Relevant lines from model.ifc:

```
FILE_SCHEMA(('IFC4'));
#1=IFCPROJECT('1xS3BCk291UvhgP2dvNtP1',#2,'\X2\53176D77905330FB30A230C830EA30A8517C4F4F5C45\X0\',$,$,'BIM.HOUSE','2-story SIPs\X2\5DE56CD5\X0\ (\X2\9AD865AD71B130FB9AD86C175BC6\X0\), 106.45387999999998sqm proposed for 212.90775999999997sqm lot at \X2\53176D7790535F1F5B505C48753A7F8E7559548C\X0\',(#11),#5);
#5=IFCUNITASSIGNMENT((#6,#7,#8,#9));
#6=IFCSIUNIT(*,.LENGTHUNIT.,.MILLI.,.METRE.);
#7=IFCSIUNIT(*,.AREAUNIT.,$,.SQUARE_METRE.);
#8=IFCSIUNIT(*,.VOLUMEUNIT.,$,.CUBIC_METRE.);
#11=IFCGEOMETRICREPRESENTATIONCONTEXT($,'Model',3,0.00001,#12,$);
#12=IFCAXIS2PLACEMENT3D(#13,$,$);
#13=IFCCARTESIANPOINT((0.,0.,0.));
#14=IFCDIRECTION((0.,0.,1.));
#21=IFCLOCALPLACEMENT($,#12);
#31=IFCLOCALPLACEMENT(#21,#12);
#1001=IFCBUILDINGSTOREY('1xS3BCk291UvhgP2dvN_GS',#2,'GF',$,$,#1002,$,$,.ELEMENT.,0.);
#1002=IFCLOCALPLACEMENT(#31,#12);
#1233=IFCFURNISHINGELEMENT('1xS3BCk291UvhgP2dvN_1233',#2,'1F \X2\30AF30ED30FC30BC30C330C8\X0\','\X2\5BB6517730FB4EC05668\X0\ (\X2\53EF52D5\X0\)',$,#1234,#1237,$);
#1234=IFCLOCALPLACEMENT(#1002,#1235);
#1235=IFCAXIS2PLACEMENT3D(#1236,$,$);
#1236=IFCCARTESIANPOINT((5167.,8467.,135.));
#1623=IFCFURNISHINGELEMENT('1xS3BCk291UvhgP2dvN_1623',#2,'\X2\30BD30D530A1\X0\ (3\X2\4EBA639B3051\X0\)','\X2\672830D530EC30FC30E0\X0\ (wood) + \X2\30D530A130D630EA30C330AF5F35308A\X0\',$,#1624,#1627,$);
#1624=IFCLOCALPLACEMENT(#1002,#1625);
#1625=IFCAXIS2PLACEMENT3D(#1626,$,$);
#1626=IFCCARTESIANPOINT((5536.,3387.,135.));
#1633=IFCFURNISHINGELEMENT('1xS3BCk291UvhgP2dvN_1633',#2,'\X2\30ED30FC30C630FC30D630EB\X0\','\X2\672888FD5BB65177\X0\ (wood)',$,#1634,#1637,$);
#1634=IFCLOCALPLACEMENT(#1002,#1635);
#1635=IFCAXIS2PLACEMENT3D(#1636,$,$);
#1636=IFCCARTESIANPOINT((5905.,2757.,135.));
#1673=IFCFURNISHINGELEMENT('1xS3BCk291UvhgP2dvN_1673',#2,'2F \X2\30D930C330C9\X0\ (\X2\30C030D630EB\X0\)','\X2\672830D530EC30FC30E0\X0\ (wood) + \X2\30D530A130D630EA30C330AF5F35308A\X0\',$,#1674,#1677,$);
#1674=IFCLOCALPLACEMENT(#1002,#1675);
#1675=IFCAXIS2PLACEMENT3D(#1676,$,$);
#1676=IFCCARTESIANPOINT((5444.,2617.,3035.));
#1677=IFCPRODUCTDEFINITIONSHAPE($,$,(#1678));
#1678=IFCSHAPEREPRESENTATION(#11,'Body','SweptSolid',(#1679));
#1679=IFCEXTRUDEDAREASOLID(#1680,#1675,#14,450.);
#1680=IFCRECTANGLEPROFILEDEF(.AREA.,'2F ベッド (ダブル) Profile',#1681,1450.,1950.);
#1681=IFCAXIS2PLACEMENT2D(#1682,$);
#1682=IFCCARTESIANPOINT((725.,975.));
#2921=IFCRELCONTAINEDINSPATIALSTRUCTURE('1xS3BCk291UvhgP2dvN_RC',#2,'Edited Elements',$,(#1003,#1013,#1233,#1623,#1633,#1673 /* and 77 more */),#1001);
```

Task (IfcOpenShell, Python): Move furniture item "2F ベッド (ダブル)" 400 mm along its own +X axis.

```python
import ifcopenshell
import ifcopenshell.api.geometry
import ifcopenshell.util.placement
import ifcopenshell.util.unit

model = ifcopenshell.open("model.ifc")
unit_scale = ifcopenshell.util.unit.calculate_unit_scale(model)

item = model.by_guid("1xS3BCk291UvhgP2dvN_1673")
matrix = ifcopenshell.util.placement.get_local_placement(item.ObjectPlacement)
matrix[:3, 3] += matrix[:3, 0] * 0.4 / unit_scale
ifcopenshell.api.geometry.edit_object_placement(model, product=item, matrix=matrix, is_si=False)

print(ifcopenshell.util.placement.get_local_placement(item.ObjectPlacement).round(3) + 0.0)

model.write("model_updated.ifc")
```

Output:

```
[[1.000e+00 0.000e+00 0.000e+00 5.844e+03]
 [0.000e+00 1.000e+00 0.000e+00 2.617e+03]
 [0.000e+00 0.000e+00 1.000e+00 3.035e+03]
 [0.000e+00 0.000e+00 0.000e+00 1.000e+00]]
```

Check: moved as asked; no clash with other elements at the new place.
